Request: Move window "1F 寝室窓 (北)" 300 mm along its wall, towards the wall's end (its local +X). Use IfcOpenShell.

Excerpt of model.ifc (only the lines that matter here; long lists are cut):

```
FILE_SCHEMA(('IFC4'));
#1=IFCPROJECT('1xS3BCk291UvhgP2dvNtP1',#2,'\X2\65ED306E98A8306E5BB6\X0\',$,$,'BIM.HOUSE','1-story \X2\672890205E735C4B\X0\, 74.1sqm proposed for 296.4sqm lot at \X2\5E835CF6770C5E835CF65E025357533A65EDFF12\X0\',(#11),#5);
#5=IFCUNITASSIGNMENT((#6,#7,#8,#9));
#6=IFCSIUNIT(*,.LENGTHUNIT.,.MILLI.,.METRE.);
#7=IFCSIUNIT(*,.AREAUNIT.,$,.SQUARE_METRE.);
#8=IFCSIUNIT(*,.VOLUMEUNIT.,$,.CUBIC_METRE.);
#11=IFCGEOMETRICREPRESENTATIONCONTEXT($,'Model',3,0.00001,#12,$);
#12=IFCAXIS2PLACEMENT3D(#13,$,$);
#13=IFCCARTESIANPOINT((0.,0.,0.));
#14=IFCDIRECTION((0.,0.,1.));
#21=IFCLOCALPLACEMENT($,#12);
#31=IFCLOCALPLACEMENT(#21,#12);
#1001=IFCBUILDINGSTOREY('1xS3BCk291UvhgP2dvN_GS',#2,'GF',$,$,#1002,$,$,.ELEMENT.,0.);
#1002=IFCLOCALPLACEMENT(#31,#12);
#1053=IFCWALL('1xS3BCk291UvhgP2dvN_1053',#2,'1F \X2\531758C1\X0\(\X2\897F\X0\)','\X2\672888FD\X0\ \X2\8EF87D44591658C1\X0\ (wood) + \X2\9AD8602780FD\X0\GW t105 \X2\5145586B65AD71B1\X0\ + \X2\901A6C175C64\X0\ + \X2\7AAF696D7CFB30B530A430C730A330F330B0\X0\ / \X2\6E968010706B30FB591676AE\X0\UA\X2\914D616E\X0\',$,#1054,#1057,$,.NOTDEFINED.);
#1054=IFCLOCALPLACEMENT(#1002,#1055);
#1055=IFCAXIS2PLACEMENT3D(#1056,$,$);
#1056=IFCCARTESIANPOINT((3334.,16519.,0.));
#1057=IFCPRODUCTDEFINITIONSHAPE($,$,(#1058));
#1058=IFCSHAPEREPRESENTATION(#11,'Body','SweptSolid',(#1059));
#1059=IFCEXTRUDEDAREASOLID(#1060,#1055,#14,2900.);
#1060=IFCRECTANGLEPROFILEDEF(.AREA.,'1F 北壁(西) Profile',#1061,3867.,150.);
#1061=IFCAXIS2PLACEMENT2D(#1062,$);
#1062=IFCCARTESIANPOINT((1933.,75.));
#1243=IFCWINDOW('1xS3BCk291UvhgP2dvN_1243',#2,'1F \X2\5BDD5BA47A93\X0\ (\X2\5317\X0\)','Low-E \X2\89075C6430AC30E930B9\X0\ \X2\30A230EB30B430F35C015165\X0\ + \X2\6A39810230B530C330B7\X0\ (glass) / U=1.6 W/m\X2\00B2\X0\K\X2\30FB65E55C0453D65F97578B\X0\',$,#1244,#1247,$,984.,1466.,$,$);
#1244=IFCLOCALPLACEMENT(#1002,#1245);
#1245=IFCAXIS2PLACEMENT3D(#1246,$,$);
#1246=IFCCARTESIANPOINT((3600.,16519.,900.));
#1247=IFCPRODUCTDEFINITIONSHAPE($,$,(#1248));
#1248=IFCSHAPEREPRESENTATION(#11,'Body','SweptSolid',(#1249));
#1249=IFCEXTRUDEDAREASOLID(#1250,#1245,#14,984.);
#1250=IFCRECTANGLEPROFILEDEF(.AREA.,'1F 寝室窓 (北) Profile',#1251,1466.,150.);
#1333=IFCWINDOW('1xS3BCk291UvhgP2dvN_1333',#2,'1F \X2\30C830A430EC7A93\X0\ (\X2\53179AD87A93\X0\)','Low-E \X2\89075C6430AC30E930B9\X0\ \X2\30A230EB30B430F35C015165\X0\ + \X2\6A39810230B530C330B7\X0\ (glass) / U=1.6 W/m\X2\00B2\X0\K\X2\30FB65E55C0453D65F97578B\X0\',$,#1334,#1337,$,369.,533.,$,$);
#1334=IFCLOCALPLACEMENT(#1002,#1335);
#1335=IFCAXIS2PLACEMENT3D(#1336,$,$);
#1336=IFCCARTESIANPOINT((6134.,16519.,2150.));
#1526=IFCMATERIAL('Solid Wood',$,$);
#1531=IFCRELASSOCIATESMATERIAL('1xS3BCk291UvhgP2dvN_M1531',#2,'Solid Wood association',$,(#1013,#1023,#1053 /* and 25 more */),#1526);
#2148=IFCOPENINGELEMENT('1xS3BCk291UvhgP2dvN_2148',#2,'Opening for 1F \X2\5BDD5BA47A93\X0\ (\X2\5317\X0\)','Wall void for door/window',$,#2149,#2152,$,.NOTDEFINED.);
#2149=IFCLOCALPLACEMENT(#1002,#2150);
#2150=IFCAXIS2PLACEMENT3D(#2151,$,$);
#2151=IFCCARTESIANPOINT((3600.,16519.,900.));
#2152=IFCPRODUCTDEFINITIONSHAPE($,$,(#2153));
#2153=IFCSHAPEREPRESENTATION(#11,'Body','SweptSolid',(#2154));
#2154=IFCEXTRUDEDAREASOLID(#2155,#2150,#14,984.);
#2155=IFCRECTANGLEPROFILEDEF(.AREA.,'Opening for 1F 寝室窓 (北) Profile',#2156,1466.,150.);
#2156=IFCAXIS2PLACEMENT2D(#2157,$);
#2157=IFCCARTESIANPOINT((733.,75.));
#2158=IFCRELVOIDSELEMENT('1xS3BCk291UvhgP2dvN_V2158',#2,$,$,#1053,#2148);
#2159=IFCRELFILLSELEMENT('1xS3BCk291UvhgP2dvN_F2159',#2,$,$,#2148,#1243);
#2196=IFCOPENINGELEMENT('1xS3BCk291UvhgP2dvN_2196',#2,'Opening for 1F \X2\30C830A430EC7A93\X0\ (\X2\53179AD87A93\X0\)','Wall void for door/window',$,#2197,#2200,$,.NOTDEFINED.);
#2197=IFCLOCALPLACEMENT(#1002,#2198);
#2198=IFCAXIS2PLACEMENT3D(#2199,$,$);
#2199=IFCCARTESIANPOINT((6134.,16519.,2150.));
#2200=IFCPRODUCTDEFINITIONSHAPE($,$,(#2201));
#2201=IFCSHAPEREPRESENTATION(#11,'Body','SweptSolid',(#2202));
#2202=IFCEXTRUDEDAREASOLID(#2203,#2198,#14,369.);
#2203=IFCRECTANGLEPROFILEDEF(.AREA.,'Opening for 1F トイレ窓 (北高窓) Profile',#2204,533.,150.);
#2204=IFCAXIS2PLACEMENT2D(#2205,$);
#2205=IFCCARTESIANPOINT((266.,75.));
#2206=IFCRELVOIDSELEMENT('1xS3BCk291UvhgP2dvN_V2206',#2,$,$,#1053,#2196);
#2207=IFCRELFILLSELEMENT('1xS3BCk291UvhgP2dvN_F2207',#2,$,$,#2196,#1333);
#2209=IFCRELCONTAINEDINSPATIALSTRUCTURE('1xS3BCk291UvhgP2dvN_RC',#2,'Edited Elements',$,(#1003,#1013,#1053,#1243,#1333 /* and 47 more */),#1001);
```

```python
import ifcopenshell
import ifcopenshell.api.geometry
import ifcopenshell.util.placement
import ifcopenshell.util.unit

model = ifcopenshell.open("model.ifc")
unit_scale = ifcopenshell.util.unit.calculate_unit_scale(model)

window = model.by_guid("1xS3BCk291UvhgP2dvN_1243")
opening = window.FillsVoids[0].RelatingOpeningElement
wall = opening.VoidsElements[0].RelatingBuildingElement

wall_matrix = ifcopenshell.util.placement.get_local_placement(wall.ObjectPlacement)
shift = wall_matrix[:3, 0] * 0.3 / unit_scale
before = ifcopenshell.util.placement.get_local_placement(window.ObjectPlacement)[:3, 3].copy()

# The window is not placed relative to its opening, so move both.
for product in (opening, window):
    matrix = ifcopenshell.util.placement.get_local_placement(product.ObjectPlacement)
    matrix[:3, 3] += shift
    ifcopenshell.api.geometry.edit_object_placement(model, product=product, matrix=matrix, is_si=False)

after = ifcopenshell.util.placement.get_local_placement(window.ObjectPlacement)[:3, 3]
print("window moved by", (after - before).round(3) + 0.0)

model.write("model-out.ifc")
```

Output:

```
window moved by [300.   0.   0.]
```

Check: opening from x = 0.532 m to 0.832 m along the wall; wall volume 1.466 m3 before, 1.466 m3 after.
